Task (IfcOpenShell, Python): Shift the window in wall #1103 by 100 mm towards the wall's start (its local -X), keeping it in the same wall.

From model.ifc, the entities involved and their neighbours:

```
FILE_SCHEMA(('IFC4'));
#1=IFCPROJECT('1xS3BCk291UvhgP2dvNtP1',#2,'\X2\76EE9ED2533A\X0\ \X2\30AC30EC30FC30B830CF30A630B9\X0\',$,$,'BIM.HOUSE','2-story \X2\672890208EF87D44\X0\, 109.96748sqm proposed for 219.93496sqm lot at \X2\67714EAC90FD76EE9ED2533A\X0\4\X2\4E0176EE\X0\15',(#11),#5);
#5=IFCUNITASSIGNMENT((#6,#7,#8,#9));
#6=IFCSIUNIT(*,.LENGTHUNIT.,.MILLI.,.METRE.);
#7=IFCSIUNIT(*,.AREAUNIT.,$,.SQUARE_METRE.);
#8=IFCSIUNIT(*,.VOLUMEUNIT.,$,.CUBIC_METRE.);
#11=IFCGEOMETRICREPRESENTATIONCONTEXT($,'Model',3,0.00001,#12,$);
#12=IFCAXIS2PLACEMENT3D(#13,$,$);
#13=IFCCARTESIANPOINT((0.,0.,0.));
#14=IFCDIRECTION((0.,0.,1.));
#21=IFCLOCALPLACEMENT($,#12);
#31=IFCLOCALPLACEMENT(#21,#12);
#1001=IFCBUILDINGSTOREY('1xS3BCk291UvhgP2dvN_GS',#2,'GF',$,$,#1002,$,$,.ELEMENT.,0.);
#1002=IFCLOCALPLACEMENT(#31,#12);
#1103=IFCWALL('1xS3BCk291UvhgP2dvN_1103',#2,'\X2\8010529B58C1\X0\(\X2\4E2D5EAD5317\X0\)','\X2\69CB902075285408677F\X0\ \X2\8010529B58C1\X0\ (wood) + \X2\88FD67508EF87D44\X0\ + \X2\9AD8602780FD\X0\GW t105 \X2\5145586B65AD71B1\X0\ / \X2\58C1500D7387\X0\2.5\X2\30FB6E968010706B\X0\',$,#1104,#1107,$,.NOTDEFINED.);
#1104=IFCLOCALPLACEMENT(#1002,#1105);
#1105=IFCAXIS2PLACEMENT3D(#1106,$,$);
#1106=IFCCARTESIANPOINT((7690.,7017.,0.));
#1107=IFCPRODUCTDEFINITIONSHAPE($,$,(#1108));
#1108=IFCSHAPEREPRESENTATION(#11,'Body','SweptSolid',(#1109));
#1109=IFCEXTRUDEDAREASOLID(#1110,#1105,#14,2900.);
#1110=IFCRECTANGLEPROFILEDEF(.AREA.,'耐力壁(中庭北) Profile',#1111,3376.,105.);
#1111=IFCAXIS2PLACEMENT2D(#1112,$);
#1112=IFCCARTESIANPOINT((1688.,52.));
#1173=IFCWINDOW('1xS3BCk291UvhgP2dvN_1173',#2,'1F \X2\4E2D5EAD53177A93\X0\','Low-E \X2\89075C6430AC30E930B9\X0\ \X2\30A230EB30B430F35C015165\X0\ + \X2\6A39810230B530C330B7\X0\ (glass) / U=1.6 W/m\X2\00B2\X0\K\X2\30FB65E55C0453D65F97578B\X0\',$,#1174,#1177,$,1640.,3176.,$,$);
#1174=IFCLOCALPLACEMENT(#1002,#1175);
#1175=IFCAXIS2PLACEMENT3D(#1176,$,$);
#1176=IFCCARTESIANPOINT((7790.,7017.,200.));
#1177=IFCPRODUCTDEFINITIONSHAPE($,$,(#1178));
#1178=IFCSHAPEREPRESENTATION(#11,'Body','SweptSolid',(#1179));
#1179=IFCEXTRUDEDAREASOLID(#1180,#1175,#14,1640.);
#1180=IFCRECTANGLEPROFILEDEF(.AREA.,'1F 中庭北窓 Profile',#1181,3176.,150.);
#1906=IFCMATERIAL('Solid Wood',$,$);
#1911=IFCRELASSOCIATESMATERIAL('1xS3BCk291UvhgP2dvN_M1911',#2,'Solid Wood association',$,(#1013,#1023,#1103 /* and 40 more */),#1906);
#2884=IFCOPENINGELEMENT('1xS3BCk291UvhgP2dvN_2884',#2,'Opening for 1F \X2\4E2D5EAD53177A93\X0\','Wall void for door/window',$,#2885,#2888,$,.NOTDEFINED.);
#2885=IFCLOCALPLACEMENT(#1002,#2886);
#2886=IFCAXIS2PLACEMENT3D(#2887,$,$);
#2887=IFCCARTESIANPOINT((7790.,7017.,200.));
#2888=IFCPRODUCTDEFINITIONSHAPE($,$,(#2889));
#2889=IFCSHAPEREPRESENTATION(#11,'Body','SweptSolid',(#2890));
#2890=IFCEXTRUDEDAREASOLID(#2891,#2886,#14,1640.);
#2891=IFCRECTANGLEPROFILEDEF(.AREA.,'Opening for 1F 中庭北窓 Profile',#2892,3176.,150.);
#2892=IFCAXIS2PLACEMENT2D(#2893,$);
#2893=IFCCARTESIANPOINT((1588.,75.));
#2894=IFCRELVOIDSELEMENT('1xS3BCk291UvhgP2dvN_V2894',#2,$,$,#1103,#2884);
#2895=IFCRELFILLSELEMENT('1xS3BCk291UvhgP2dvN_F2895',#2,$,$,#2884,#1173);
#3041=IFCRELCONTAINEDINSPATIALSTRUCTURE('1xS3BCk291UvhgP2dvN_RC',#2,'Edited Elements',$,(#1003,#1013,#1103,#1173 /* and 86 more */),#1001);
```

```python
import ifcopenshell
import ifcopenshell.api.geometry
import ifcopenshell.util.placement

model = ifcopenshell.open("model.ifc")

window = model.by_guid("1xS3BCk291UvhgP2dvN_1173")
opening = window.FillsVoids[0].RelatingOpeningElement
wall = opening.VoidsElements[0].RelatingBuildingElement

wall_matrix = ifcopenshell.util.placement.get_local_placement(wall.ObjectPlacement)
shift = wall_matrix[:3, 0] * -100.0
before = ifcopenshell.util.placement.get_local_placement(window.ObjectPlacement)[:3, 3].copy()

# The window is not placed relative to its opening, so move both.
for product in (opening, window):
    matrix = ifcopenshell.util.placement.get_local_placement(product.ObjectPlacement)
    matrix[:3, 3] += shift
    ifcopenshell.api.geometry.edit_object_placement(model, product=product, matrix=matrix, is_si=False)

after = ifcopenshell.util.placement.get_local_placement(window.ObjectPlacement)[:3, 3]
print("window moved by", (after - before).round(3) + 0.0)

model.write("model_rev.ifc")
```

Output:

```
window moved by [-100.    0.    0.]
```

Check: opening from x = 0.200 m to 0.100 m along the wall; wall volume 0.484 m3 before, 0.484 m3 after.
